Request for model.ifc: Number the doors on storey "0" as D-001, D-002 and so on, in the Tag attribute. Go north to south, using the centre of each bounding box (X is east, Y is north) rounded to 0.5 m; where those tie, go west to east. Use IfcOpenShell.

First a look at what the model holds.

```python
import ifcopenshell
import ifcopenshell.util.element
import ifcopenshell.util.placement

model = ifcopenshell.open("model.ifc")
print(model.schema)
storey = next(s for s in model.by_type("IfcBuildingStorey") if s.Name == "0")
doors = [e for e in ifcopenshell.util.element.get_decomposition(storey) if e.is_a("IfcDoor")]
for e in sorted(doors, key=lambda e: e.id()):
    origin = ifcopenshell.util.placement.get_local_placement(e.ObjectPlacement)[:3, 3]
    print(e.id(), e.Tag, e.Name, origin.round(2) + 0.0, sep=" | ")
```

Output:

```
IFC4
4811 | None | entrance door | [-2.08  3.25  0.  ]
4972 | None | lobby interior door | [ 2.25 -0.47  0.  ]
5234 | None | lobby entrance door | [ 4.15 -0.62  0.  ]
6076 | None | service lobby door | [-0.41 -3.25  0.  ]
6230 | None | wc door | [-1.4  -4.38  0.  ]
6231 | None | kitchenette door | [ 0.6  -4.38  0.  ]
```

```python
import ifcopenshell
import ifcopenshell.geom
import ifcopenshell.util.element
import ifcopenshell.util.shape

model = ifcopenshell.open("model.ifc")
settings = ifcopenshell.geom.settings()
settings.set("use-world-coords", True)


def centre(element):
    shape = ifcopenshell.geom.create_shape(settings, element)
    return ifcopenshell.util.shape.get_bbox_centroid(shape.geometry)


storey = next(s for s in model.by_type("IfcBuildingStorey") if s.Name == "0")
doors = [e for e in ifcopenshell.util.element.get_decomposition(storey) if e.is_a("IfcDoor")]

# Insertion points can sit at a corner or the storey origin, so sort by the geometry (in metres).
centres = {e: centre(e) for e in doors}
doors.sort(key=lambda e: (-round(centres[e][1] / 0.5), centres[e][0]))

for i, e in enumerate(doors, start=1):
    number = f"D-0{i:02d}"
    e.Tag = number
    print(e.id(), number)

model.write("model-out.ifc")
```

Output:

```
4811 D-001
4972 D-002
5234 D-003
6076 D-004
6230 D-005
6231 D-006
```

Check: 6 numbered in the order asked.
